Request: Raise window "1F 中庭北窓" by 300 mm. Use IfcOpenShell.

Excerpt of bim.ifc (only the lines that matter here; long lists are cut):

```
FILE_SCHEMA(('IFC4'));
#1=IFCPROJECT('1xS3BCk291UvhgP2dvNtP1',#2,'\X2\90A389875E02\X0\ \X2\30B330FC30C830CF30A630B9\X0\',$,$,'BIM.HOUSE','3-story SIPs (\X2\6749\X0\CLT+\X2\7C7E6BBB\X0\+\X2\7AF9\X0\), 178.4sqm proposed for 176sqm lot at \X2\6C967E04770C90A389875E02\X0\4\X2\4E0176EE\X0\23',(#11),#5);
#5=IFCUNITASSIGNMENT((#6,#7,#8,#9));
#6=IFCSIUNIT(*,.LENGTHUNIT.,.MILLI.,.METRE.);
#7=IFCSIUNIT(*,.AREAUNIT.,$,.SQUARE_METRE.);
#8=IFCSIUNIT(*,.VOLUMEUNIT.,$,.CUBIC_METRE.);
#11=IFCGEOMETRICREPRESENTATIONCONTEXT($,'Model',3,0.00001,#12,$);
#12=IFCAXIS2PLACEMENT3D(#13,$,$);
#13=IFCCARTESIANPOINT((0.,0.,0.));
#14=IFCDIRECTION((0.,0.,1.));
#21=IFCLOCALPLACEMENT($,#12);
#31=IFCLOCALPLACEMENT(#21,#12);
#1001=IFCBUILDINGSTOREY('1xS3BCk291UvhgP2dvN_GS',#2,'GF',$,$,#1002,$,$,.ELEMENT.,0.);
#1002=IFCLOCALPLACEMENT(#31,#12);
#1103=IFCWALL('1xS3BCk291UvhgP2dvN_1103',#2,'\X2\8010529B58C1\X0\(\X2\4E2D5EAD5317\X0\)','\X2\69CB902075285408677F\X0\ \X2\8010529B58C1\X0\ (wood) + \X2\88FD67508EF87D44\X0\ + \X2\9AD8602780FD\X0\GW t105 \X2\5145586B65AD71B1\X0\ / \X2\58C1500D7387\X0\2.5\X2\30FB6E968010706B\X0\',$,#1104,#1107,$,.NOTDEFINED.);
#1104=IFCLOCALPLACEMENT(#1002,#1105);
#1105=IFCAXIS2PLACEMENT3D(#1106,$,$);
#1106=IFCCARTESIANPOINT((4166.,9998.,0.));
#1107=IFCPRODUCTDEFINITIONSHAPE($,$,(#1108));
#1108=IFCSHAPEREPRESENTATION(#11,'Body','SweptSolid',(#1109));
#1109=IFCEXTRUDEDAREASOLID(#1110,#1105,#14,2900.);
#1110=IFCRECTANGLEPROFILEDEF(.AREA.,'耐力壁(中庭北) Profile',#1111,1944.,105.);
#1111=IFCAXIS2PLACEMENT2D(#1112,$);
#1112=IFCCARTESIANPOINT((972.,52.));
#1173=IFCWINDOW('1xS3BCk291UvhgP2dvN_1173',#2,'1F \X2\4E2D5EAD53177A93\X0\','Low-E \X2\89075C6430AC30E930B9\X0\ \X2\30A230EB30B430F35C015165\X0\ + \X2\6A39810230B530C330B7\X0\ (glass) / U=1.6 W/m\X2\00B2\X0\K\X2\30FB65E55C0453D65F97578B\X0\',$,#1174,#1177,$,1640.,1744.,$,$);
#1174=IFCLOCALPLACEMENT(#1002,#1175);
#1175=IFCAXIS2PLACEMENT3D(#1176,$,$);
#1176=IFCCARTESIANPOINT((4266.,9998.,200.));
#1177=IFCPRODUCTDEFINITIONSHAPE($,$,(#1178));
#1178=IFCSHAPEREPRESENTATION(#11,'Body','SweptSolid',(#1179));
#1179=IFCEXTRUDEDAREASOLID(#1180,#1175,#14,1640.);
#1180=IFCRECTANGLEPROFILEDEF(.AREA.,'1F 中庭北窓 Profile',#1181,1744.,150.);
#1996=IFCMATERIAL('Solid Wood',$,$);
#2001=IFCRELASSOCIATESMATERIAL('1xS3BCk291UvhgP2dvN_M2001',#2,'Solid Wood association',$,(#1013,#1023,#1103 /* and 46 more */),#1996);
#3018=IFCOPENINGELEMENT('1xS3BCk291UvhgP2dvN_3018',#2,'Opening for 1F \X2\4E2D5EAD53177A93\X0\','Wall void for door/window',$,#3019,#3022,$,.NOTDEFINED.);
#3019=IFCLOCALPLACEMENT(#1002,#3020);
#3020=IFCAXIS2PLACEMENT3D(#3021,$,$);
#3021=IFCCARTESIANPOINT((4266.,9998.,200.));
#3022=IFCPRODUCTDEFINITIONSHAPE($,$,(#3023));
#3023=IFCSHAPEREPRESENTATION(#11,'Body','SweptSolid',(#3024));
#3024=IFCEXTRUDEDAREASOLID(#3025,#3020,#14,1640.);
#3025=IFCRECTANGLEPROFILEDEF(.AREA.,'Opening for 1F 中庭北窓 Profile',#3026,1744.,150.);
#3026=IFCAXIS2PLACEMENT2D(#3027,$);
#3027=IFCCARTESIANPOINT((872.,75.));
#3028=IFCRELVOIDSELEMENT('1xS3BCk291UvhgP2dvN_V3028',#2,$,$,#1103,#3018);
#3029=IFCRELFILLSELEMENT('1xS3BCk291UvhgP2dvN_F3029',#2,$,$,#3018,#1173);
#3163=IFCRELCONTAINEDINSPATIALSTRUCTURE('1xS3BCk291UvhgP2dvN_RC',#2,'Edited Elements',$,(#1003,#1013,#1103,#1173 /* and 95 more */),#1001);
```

```python
import numpy as np
import ifcopenshell
import ifcopenshell.api.geometry
import ifcopenshell.util.placement
import ifcopenshell.util.unit

model = ifcopenshell.open("bim.ifc")
unit_scale = ifcopenshell.util.unit.calculate_unit_scale(model)

window = model.by_guid("1xS3BCk291UvhgP2dvN_1173")
opening = window.FillsVoids[0].RelatingOpeningElement
dz = 300.0

shift = np.array([0.0, 0.0, dz])
# The window is not placed relative to its opening, so move both.
for product in (opening, window):
    matrix = ifcopenshell.util.placement.get_local_placement(product.ObjectPlacement)
    matrix[:3, 3] += shift
    ifcopenshell.api.geometry.edit_object_placement(model, product=product, matrix=matrix, is_si=False)

print(f"moved by {dz * unit_scale:+.3f} m")

model.write("bim_updated.ifc")
```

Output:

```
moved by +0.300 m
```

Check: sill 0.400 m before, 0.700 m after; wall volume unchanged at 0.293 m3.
